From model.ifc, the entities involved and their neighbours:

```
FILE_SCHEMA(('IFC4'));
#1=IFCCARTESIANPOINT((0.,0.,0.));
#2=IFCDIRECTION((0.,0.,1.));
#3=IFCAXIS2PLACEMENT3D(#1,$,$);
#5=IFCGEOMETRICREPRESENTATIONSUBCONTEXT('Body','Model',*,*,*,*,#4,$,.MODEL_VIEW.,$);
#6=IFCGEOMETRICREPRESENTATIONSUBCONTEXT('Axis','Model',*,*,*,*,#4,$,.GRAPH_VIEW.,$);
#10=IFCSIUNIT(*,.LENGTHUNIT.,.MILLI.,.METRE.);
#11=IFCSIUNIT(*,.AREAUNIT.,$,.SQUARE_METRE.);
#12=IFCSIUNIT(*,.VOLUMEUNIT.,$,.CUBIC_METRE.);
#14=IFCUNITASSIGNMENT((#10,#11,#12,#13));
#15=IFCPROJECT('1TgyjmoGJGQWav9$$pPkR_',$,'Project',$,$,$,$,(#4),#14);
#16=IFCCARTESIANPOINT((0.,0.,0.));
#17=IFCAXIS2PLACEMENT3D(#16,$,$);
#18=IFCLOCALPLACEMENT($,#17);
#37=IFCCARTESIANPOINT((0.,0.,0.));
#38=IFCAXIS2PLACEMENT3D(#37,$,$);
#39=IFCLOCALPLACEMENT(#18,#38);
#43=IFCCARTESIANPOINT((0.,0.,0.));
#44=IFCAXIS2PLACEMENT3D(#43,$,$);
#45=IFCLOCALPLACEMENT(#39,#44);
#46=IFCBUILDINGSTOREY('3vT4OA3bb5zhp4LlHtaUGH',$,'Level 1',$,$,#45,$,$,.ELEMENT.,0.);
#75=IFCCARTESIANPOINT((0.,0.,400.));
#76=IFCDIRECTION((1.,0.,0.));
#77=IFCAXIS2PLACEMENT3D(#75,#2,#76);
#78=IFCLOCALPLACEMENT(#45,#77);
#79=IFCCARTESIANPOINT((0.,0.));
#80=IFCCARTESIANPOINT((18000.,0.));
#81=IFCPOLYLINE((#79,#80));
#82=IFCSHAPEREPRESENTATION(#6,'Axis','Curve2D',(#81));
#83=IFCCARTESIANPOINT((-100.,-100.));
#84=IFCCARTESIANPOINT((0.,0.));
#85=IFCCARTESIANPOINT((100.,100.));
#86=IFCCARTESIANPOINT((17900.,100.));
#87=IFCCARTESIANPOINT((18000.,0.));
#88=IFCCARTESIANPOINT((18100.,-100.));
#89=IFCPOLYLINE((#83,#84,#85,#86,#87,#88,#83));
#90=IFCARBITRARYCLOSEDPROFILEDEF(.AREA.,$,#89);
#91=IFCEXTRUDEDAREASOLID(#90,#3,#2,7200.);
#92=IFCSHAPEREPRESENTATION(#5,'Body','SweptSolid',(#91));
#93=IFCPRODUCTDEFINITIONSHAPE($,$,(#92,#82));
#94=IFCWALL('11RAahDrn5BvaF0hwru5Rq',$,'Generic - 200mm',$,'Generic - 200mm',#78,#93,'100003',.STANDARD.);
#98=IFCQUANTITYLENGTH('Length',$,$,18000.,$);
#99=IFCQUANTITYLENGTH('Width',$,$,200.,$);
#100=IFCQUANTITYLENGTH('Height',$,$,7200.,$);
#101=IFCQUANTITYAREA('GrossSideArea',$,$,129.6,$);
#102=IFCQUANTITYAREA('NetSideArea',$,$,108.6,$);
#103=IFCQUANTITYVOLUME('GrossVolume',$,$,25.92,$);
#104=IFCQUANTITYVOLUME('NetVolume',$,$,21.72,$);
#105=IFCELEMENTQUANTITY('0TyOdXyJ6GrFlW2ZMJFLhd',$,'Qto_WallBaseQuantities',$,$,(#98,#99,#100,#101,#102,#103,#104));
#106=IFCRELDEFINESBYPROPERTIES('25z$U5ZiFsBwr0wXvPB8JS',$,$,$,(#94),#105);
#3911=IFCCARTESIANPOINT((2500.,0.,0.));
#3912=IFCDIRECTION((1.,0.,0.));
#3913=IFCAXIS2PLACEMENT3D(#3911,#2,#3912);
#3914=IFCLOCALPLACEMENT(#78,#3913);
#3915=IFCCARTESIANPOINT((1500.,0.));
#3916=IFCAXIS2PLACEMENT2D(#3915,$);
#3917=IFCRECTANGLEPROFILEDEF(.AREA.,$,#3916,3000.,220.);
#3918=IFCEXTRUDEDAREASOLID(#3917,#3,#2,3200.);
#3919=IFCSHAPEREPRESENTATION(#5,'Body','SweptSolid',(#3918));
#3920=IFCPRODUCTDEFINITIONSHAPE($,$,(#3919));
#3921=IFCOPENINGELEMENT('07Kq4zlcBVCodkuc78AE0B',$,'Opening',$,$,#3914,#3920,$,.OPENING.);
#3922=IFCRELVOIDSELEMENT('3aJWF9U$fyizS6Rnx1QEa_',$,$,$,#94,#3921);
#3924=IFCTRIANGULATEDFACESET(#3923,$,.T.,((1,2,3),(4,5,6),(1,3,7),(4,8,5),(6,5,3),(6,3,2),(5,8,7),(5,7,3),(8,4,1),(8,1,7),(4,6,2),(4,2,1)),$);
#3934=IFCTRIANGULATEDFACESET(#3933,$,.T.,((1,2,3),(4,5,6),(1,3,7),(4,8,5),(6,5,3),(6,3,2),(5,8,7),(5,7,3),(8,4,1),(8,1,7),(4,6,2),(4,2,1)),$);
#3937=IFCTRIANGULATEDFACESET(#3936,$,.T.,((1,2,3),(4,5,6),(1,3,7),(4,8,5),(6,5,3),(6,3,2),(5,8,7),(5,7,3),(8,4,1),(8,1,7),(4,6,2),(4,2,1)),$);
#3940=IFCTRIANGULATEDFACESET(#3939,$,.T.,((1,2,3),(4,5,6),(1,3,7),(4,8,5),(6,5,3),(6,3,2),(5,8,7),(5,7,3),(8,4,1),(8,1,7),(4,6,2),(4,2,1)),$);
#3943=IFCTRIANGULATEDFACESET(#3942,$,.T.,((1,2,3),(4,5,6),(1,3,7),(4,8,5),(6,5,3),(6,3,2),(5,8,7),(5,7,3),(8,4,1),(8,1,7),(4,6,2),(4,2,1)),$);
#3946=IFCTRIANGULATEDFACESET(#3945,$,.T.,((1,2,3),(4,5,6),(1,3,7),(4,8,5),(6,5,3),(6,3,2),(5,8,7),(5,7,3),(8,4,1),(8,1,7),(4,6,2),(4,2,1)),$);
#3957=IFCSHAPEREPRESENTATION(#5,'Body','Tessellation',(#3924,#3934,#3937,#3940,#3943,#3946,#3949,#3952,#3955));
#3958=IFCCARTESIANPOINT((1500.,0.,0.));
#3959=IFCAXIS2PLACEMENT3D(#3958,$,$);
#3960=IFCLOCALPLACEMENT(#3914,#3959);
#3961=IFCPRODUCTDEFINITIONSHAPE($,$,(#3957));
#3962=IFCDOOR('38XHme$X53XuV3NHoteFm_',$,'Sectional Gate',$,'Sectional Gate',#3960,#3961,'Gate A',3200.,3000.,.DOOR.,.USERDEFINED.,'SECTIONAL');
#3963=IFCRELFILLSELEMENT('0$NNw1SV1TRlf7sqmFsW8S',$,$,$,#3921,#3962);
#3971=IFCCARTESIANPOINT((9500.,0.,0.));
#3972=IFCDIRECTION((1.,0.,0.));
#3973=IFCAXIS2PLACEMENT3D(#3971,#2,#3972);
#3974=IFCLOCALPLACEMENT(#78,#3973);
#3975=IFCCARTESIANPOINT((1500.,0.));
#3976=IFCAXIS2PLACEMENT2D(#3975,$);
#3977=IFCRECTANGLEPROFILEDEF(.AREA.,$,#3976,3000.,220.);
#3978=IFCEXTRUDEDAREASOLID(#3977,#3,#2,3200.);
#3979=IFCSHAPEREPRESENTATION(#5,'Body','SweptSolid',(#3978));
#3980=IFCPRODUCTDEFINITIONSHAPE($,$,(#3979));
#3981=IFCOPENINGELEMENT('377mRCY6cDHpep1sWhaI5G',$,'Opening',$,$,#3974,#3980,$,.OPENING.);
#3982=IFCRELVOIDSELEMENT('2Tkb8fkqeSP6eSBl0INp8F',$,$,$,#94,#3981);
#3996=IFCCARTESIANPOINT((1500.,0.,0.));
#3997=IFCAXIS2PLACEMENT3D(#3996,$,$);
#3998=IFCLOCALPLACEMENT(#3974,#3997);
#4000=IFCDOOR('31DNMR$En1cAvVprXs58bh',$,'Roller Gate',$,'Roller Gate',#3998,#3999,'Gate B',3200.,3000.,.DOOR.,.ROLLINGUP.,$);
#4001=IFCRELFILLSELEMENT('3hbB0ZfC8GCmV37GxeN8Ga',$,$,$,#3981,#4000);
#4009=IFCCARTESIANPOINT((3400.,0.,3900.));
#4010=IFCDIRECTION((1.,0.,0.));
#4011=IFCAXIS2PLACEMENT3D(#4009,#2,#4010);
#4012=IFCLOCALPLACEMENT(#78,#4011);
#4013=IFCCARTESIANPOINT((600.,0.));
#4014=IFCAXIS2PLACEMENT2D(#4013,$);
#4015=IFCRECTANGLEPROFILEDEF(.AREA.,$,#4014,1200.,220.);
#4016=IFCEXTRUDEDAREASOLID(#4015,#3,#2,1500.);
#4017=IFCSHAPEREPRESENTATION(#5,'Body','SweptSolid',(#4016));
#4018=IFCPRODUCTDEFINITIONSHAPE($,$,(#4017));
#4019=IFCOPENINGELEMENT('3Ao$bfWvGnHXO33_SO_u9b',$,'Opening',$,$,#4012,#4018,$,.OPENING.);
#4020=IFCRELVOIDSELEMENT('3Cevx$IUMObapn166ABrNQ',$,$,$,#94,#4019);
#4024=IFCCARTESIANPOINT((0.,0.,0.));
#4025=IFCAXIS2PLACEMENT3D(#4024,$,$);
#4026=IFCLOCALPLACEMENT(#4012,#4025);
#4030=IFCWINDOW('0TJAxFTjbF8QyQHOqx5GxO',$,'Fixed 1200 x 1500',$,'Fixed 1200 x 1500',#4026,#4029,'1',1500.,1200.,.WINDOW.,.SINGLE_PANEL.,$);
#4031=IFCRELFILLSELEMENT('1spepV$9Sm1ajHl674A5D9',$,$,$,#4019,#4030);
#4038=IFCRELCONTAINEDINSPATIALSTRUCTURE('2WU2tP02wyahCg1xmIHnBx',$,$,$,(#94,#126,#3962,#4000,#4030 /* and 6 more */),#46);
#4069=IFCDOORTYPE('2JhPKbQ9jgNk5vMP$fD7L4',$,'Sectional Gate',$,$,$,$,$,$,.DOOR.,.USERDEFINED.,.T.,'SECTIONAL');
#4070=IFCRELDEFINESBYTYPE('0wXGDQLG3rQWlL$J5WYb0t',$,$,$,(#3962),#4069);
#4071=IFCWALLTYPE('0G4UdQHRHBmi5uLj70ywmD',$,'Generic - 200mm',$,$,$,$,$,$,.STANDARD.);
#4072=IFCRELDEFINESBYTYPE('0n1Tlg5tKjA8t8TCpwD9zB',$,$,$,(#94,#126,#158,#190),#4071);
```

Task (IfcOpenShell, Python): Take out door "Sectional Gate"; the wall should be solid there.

```python
import ifcopenshell
import ifcopenshell.api.feature
import ifcopenshell.api.pset
import ifcopenshell.api.root
import ifcopenshell.geom
import ifcopenshell.util.element
import ifcopenshell.util.shape
import ifcopenshell.util.unit

model = ifcopenshell.open("model.ifc")
area_scale = ifcopenshell.util.unit.calculate_unit_scale(model, "AREAUNIT")
volume_scale = ifcopenshell.util.unit.calculate_unit_scale(model, "VOLUMEUNIT")
settings = ifcopenshell.geom.settings()


def volume(element):
    """Net volume in cubic metres, openings subtracted."""
    shape = ifcopenshell.geom.create_shape(settings, element)
    return ifcopenshell.util.shape.get_volume(shape.geometry)


door = model.by_id(3962)
opening = door.FillsVoids[0].RelatingOpeningElement
wall = opening.VoidsElements[0].RelatingBuildingElement
before = volume(wall)

ifcopenshell.api.root.remove_product(model, product=door)
ifcopenshell.api.feature.remove_feature(model, feature=opening)

after = volume(wall)
thickness = 0.2  # wall thickness in metres

# Update the wall's stored quantities.
qto = model.by_id(ifcopenshell.util.element.get_pset(wall, "Qto_WallBaseQuantities", should_inherit=False)["id"])
ifcopenshell.api.pset.edit_qto(model, qto=qto, properties={
    "NetSideArea": after / thickness / area_scale,
    "NetVolume": after / volume_scale,
})

print(f"wall volume {before:.3f} -> {after:.3f} m3")

model.write("model_edited.ifc")
```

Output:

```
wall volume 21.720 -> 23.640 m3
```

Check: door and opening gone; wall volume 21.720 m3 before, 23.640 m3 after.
